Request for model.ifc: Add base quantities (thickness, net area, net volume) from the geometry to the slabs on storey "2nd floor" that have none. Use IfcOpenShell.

First a look at what the model holds.

```python
import ifcopenshell
import ifcopenshell.util.element
import ifcopenshell.util.unit

model = ifcopenshell.open("model.ifc")
print(model.schema)
for unit_type in ("LENGTHUNIT", "AREAUNIT", "VOLUMEUNIT"):
    print(unit_type, ifcopenshell.util.unit.calculate_unit_scale(model, unit_type))
storey = next(s for s in model.by_type("IfcBuildingStorey") if s.Name == "2nd floor")
slabs = [e for e in ifcopenshell.util.element.get_decomposition(storey) if e.is_a("IfcSlab")]
for e in sorted(slabs, key=lambda e: e.id()):
    print(e.id(), e.is_a(), e.Name, list(ifcopenshell.util.element.get_psets(e, qtos_only=True)), sep=" | ")
```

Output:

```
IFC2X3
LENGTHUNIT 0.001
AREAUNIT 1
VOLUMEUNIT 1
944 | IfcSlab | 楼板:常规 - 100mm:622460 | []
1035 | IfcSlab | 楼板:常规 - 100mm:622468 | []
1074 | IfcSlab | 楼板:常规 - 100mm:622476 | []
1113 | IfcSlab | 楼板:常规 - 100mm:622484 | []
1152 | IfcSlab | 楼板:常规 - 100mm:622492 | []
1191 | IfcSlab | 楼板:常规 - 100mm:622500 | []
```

```python
import ifcopenshell
import ifcopenshell.api.pset
import ifcopenshell.geom
import ifcopenshell.util.element
import ifcopenshell.util.shape
import ifcopenshell.util.unit

model = ifcopenshell.open("model.ifc")
unit_scale = ifcopenshell.util.unit.calculate_unit_scale(model)
area_scale = ifcopenshell.util.unit.calculate_unit_scale(model, "AREAUNIT")
volume_scale = ifcopenshell.util.unit.calculate_unit_scale(model, "VOLUMEUNIT")
settings = ifcopenshell.geom.settings()

storey = next(s for s in model.by_type("IfcBuildingStorey") if s.Name == "2nd floor")
slabs = [e for e in ifcopenshell.util.element.get_decomposition(storey) if e.is_a("IfcSlab")]

for e in sorted(slabs, key=lambda e: e.id()):
    if ifcopenshell.util.element.get_psets(e, qtos_only=True, should_inherit=False):
        continue
    # Geometry comes back in metres, in the element's own axes.
    shape = ifcopenshell.geom.create_shape(settings, e)
    values = {
        "Width": ifcopenshell.util.shape.get_z(shape.geometry) / unit_scale,
        "NetArea": ifcopenshell.util.shape.get_footprint_area(shape.geometry) / area_scale,
        "NetVolume": ifcopenshell.util.shape.get_volume(shape.geometry) / volume_scale,
    }
    qto = ifcopenshell.api.pset.add_qto(model, product=e, name="BaseQuantities")
    ifcopenshell.api.pset.edit_qto(model, qto=qto, properties=values)
    print(e.id(), {k: round(v, 3) for k, v in values.items()})

model.write("model_rev.ifc")
```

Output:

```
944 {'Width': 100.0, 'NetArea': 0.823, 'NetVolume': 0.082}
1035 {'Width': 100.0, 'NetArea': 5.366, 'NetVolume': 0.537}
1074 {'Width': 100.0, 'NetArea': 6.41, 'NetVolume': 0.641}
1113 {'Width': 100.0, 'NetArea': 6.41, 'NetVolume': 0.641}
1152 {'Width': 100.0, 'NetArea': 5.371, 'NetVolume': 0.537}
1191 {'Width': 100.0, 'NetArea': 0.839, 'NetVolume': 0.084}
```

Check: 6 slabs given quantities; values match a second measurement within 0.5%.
